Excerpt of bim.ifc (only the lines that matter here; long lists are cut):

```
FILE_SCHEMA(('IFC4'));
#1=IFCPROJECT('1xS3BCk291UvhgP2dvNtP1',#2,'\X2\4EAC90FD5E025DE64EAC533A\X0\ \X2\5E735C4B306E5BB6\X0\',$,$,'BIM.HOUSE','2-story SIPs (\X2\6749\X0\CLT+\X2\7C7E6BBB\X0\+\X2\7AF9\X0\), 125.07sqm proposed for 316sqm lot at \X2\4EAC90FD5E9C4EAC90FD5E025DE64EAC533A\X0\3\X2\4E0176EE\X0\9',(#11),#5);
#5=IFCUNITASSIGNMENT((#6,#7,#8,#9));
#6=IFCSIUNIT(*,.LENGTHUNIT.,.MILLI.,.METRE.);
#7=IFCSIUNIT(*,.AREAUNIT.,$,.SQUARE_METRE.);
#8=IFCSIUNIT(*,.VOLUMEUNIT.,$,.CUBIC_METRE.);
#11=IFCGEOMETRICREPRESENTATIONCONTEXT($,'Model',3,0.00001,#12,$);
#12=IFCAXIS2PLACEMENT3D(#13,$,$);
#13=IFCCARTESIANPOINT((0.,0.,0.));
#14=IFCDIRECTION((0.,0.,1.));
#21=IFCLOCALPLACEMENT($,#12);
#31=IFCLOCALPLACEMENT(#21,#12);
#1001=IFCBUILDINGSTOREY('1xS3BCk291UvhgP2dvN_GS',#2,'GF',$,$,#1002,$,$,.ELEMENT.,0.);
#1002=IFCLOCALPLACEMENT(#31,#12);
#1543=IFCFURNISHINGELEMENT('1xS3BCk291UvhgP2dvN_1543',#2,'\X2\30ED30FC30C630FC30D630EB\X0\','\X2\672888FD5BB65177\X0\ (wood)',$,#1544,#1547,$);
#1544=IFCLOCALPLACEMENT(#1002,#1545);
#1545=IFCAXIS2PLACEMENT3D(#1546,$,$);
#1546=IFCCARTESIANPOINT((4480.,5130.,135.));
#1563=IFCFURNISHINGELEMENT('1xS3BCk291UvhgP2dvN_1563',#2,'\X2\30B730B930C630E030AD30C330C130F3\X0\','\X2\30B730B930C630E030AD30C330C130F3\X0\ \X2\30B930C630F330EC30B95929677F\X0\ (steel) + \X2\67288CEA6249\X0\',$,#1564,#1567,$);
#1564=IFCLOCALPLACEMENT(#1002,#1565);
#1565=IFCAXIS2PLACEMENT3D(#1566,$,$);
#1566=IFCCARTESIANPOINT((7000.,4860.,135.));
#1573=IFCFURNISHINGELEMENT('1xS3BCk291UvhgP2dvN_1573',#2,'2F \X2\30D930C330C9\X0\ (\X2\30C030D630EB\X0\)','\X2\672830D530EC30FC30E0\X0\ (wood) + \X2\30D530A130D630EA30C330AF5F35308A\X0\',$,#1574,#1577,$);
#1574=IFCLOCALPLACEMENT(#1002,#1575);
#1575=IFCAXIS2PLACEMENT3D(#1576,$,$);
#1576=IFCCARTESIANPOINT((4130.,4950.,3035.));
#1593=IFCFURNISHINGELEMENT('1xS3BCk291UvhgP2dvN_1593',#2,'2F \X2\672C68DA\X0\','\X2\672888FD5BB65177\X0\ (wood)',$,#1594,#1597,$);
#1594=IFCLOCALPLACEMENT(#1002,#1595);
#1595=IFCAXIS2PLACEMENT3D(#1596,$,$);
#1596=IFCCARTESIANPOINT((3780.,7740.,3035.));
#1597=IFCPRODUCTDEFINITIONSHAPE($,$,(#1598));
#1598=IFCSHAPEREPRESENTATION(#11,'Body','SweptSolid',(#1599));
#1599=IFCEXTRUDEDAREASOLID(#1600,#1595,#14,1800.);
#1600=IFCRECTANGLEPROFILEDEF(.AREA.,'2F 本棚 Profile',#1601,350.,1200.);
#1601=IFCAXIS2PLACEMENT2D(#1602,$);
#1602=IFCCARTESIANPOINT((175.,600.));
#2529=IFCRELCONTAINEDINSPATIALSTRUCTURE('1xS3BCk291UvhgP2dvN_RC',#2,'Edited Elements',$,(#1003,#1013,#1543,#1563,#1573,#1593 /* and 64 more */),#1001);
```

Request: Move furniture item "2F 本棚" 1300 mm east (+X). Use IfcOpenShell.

```python
import ifcopenshell
import ifcopenshell.api.geometry
import ifcopenshell.util.placement
import ifcopenshell.util.unit

model = ifcopenshell.open("bim.ifc")
unit_scale = ifcopenshell.util.unit.calculate_unit_scale(model)

item = model.by_guid("1xS3BCk291UvhgP2dvN_1593")
matrix = ifcopenshell.util.placement.get_local_placement(item.ObjectPlacement)
matrix[0, 3] += 1.3 / unit_scale
ifcopenshell.api.geometry.edit_object_placement(model, product=item, matrix=matrix, is_si=False)

print(ifcopenshell.util.placement.get_local_placement(item.ObjectPlacement).round(3) + 0.0)

model.write("bim_edited.ifc")
```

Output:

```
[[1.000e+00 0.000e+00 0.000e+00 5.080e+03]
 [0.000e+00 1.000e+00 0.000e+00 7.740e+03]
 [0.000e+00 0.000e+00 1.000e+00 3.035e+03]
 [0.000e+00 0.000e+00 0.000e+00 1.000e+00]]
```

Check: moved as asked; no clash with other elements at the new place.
